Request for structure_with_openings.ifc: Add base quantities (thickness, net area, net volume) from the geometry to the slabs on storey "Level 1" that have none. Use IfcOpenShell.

First a look at what the model holds.

```python
import ifcopenshell
import ifcopenshell.util.element
import ifcopenshell.util.unit

model = ifcopenshell.open("structure_with_openings.ifc")
print(model.schema)
for unit_type in ("LENGTHUNIT", "AREAUNIT", "VOLUMEUNIT"):
    print(unit_type, ifcopenshell.util.unit.calculate_unit_scale(model, unit_type))
storey = next(s for s in model.by_type("IfcBuildingStorey") if s.Name == "Level 1")
slabs = [e for e in ifcopenshell.util.element.get_decomposition(storey) if e.is_a("IfcSlab")]
for e in sorted(slabs, key=lambda e: e.id()):
    print(e.id(), e.is_a(), e.Name, list(ifcopenshell.util.element.get_psets(e, qtos_only=True)), sep=" | ")
```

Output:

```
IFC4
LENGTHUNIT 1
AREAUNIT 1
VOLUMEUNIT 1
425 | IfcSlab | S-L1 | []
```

```python
import ifcopenshell
import ifcopenshell.api.pset
import ifcopenshell.geom
import ifcopenshell.util.element
import ifcopenshell.util.shape
import ifcopenshell.util.unit

model = ifcopenshell.open("structure_with_openings.ifc")
unit_scale = ifcopenshell.util.unit.calculate_unit_scale(model)
area_scale = ifcopenshell.util.unit.calculate_unit_scale(model, "AREAUNIT")
volume_scale = ifcopenshell.util.unit.calculate_unit_scale(model, "VOLUMEUNIT")
settings = ifcopenshell.geom.settings()

storey = next(s for s in model.by_type("IfcBuildingStorey") if s.Name == "Level 1")
slabs = [e for e in ifcopenshell.util.element.get_decomposition(storey) if e.is_a("IfcSlab")]

for e in sorted(slabs, key=lambda e: e.id()):
    if ifcopenshell.util.element.get_psets(e, qtos_only=True, should_inherit=False):
        continue
    # Geometry comes back in metres, in the element's own axes.
    shape = ifcopenshell.geom.create_shape(settings, e)
    values = {
        "Width": ifcopenshell.util.shape.get_z(shape.geometry) / unit_scale,
        "NetArea": ifcopenshell.util.shape.get_footprint_area(shape.geometry) / area_scale,
        "NetVolume": ifcopenshell.util.shape.get_volume(shape.geometry) / volume_scale,
    }
    qto = ifcopenshell.api.pset.add_qto(model, product=e, name="Qto_SlabBaseQuantities")
    ifcopenshell.api.pset.edit_qto(model, qto=qto, properties=values)
    print(e.id(), {k: round(v, 3) for k, v in values.items()})

model.write("structure_with_openings_rev.ifc")
```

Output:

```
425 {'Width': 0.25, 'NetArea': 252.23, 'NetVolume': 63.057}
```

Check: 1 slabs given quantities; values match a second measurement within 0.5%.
